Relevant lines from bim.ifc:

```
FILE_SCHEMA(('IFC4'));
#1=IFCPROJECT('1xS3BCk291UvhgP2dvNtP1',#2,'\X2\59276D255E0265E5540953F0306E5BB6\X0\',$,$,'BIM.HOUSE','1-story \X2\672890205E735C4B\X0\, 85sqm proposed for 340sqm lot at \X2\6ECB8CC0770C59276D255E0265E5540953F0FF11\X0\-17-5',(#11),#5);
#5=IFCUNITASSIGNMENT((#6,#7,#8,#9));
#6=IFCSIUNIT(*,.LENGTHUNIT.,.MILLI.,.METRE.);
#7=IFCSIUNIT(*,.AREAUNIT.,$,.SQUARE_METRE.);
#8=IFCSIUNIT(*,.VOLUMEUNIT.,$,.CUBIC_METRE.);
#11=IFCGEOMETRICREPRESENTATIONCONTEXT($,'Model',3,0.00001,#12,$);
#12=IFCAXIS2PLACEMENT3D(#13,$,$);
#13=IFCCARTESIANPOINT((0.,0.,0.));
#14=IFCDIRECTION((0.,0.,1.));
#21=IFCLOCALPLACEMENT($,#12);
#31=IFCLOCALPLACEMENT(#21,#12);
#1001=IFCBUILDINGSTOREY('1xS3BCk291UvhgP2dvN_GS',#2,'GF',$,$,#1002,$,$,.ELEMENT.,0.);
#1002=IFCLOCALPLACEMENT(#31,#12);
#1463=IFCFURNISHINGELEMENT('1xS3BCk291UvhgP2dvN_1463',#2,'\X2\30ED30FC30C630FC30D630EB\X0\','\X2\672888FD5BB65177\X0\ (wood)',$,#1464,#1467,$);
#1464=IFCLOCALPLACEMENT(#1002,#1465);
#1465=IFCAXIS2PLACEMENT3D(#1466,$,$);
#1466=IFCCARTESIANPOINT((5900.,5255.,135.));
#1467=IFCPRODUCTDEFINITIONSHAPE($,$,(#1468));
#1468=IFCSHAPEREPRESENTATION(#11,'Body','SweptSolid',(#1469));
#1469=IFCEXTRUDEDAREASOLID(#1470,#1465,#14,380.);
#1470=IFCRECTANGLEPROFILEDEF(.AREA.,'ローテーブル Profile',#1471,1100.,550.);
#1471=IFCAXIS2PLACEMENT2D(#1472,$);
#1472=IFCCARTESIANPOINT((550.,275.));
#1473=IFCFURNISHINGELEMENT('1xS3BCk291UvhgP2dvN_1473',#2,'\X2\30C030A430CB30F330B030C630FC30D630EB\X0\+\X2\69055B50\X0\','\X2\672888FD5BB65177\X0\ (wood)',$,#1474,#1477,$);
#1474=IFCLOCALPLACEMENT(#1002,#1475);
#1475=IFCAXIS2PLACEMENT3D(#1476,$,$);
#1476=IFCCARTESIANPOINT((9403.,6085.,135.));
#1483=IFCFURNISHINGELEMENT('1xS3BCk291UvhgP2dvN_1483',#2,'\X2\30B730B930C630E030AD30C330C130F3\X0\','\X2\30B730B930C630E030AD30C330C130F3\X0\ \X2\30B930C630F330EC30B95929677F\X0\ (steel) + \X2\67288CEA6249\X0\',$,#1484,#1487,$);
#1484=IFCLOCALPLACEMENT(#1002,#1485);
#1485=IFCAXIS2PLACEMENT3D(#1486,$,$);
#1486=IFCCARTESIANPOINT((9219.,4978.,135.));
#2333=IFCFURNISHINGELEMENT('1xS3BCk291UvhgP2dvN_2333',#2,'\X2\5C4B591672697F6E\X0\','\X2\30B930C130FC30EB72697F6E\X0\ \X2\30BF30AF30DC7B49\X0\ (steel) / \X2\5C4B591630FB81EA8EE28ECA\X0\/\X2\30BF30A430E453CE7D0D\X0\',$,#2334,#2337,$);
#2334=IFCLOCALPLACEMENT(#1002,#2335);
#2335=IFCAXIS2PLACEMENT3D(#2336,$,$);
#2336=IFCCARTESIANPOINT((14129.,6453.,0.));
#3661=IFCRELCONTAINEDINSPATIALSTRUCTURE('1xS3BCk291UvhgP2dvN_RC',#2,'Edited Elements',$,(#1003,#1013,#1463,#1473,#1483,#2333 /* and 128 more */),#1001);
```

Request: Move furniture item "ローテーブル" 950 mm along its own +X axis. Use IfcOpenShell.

```python
import ifcopenshell
import ifcopenshell.api.geometry
import ifcopenshell.util.placement
import ifcopenshell.util.unit

model = ifcopenshell.open("bim.ifc")
unit_scale = ifcopenshell.util.unit.calculate_unit_scale(model)

item = model.by_guid("1xS3BCk291UvhgP2dvN_1463")
matrix = ifcopenshell.util.placement.get_local_placement(item.ObjectPlacement)
matrix[:3, 3] += matrix[:3, 0] * 0.95 / unit_scale
ifcopenshell.api.geometry.edit_object_placement(model, product=item, matrix=matrix, is_si=False)

print(ifcopenshell.util.placement.get_local_placement(item.ObjectPlacement).round(3) + 0.0)

model.write("bim_updated.ifc")
```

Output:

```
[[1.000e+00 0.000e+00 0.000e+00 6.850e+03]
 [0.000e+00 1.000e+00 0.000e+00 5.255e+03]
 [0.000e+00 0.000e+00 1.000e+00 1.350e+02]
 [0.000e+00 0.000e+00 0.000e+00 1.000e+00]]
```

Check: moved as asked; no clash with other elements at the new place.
